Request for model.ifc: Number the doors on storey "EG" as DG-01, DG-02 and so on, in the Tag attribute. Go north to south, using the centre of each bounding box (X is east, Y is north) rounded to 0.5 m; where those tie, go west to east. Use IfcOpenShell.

First a look at what the model holds.

```python
import ifcopenshell
import ifcopenshell.util.element
import ifcopenshell.util.placement

model = ifcopenshell.open("model.ifc")
print(model.schema)
storey = next(s for s in model.by_type("IfcBuildingStorey") if s.Name == "EG")
doors = [e for e in ifcopenshell.util.element.get_decomposition(storey) if e.is_a("IfcDoor")]
for e in sorted(doors, key=lambda e: e.id()):
    origin = ifcopenshell.util.placement.get_local_placement(e.ObjectPlacement)[:3, 3]
    print(e.id(), e.Tag, e.Name, origin.round(2) + 0.0, sep=" | ")
```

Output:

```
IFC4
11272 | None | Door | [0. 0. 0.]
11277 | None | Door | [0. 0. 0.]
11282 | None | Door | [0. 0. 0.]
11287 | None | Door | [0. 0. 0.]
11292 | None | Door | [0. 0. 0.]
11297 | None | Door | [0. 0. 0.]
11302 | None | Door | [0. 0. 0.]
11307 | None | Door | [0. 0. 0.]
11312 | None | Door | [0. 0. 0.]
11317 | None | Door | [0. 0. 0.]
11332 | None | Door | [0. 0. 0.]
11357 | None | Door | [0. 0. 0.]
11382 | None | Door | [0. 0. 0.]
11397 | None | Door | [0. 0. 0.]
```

```python
import ifcopenshell
import ifcopenshell.geom
import ifcopenshell.util.element
import ifcopenshell.util.shape

model = ifcopenshell.open("model.ifc")
settings = ifcopenshell.geom.settings()
settings.set("use-world-coords", True)


def centre(element):
    shape = ifcopenshell.geom.create_shape(settings, element)
    return ifcopenshell.util.shape.get_bbox_centroid(shape.geometry)


storey = next(s for s in model.by_type("IfcBuildingStorey") if s.Name == "EG")
doors = [e for e in ifcopenshell.util.element.get_decomposition(storey) if e.is_a("IfcDoor")]

# Insertion points can sit at a corner or the storey origin, so sort by the geometry (in metres).
centres = {e: centre(e) for e in doors}
doors.sort(key=lambda e: (-round(centres[e][1] / 0.5), centres[e][0]))

for i, e in enumerate(doors, start=1):
    number = f"DG-{i:02d}"
    e.Tag = number
    print(e.id(), number)

model.write("model_rev.ifc")
```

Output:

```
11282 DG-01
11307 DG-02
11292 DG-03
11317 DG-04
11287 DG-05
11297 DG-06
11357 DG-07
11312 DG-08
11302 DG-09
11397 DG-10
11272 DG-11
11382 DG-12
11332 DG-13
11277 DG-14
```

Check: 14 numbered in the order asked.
